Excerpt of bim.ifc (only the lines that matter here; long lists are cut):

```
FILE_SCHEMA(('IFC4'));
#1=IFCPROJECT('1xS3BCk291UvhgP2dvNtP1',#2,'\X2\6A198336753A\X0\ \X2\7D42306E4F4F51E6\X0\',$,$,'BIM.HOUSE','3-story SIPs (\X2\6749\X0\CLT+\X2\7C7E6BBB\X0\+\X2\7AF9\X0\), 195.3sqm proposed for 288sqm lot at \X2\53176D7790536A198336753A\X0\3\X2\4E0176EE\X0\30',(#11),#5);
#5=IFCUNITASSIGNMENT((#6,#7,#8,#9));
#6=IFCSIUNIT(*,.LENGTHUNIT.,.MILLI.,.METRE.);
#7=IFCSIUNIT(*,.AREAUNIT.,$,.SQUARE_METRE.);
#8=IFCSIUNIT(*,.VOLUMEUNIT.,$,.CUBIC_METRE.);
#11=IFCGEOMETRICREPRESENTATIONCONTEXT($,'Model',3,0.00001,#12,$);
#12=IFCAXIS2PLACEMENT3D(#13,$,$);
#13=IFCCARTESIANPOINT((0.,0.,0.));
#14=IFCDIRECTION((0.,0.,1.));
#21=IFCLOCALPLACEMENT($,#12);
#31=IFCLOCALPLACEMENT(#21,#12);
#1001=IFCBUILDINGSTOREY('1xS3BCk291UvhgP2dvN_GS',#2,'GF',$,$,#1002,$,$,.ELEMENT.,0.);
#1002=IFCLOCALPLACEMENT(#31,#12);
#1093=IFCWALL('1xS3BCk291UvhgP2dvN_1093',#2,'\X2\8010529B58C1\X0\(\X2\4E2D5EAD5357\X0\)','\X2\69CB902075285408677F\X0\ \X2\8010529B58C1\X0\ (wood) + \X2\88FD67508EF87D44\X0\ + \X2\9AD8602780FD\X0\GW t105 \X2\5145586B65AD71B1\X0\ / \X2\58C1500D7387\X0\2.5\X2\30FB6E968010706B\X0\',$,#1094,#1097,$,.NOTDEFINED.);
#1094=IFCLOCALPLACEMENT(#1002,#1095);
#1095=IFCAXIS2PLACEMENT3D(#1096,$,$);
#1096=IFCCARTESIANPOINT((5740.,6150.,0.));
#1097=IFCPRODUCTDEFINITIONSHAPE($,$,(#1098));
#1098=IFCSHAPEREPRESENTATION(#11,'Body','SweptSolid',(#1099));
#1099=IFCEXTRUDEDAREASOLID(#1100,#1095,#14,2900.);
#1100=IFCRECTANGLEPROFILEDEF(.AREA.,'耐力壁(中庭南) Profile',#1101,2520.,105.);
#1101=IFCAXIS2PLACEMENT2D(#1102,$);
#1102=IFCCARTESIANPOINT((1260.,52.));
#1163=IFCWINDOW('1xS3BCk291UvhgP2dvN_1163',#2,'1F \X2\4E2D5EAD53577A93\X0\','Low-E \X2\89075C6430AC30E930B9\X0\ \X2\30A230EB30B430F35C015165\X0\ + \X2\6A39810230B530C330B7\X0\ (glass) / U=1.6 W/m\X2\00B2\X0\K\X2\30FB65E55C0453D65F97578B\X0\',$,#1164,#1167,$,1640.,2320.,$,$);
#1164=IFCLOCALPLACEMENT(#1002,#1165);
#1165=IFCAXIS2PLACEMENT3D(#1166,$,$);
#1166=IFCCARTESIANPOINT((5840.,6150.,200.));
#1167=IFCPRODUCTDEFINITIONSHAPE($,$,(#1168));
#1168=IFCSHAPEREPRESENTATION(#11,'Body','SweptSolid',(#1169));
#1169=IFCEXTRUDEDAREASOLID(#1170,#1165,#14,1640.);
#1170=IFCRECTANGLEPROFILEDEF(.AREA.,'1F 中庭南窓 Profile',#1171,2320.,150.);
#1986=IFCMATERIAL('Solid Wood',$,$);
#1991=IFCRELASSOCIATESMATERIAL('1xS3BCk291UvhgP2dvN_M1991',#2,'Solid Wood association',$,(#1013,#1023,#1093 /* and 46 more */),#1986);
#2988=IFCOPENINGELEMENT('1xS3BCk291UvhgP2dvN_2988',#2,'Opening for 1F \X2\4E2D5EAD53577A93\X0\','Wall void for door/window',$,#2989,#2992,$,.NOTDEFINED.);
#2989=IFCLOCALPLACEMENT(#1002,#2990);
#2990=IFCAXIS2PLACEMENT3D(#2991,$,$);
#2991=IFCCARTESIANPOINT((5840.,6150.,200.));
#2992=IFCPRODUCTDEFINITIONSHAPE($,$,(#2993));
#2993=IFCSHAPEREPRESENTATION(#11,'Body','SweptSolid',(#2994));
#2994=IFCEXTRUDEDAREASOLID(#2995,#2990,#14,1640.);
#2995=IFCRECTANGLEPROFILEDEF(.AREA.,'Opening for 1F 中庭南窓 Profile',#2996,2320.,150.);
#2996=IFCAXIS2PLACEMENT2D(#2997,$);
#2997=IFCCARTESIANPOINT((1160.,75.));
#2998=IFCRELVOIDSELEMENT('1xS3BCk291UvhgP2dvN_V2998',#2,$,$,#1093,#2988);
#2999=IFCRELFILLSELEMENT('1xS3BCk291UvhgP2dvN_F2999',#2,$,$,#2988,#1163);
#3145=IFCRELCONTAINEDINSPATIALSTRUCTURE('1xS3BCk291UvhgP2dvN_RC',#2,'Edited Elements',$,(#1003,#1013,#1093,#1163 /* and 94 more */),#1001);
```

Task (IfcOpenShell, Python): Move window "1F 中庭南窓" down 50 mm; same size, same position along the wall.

```python
import numpy as np
import ifcopenshell
import ifcopenshell.api.geometry
import ifcopenshell.util.placement
import ifcopenshell.util.unit

model = ifcopenshell.open("bim.ifc")
unit_scale = ifcopenshell.util.unit.calculate_unit_scale(model)

window = model.by_id(1163)
opening = window.FillsVoids[0].RelatingOpeningElement
dz = -0.05 / unit_scale

shift = np.array([0.0, 0.0, dz])
# The window is not placed relative to its opening, so move both.
for product in (opening, window):
    matrix = ifcopenshell.util.placement.get_local_placement(product.ObjectPlacement)
    matrix[:3, 3] += shift
    ifcopenshell.api.geometry.edit_object_placement(model, product=product, matrix=matrix, is_si=False)

print(f"moved by {dz * unit_scale:+.3f} m")

model.write("bim-out.ifc")
```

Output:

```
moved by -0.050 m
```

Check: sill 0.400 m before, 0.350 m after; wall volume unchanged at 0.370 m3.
